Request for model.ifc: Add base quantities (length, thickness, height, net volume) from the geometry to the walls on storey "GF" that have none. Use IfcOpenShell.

First a look at what the model holds.

```python
import ifcopenshell
import ifcopenshell.util.element
import ifcopenshell.util.unit

model = ifcopenshell.open("model.ifc")
print(model.schema)
for unit_type in ("LENGTHUNIT", "AREAUNIT", "VOLUMEUNIT"):
    print(unit_type, ifcopenshell.util.unit.calculate_unit_scale(model, unit_type))
storey = next(s for s in model.by_type("IfcBuildingStorey") if s.Name == "GF")
walls = [e for e in ifcopenshell.util.element.get_decomposition(storey) if e.is_a("IfcWall")]
for e in sorted(walls, key=lambda e: e.id()):
    print(e.id(), e.is_a(), e.Name, list(ifcopenshell.util.element.get_psets(e, qtos_only=True)), sep=" | ")
```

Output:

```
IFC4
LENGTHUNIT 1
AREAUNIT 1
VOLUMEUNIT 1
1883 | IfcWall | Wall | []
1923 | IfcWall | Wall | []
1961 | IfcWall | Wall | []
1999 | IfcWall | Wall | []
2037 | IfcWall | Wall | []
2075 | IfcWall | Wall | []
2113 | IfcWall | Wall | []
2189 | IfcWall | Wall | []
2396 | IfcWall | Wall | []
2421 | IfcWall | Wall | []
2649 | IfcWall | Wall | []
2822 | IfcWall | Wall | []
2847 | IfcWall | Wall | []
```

```python
import ifcopenshell
import ifcopenshell.api.pset
import ifcopenshell.geom
import ifcopenshell.util.element
import ifcopenshell.util.shape
import ifcopenshell.util.unit

model = ifcopenshell.open("model.ifc")
unit_scale = ifcopenshell.util.unit.calculate_unit_scale(model)
volume_scale = ifcopenshell.util.unit.calculate_unit_scale(model, "VOLUMEUNIT")
settings = ifcopenshell.geom.settings()

storey = next(s for s in model.by_type("IfcBuildingStorey") if s.Name == "GF")
walls = [e for e in ifcopenshell.util.element.get_decomposition(storey) if e.is_a("IfcWall")]

for e in sorted(walls, key=lambda e: e.id()):
    if ifcopenshell.util.element.get_psets(e, qtos_only=True, should_inherit=False):
        continue
    # Geometry comes back in metres, in the element's own axes.
    shape = ifcopenshell.geom.create_shape(settings, e)
    values = {
        "Length": ifcopenshell.util.shape.get_x(shape.geometry) / unit_scale,
        "Width": ifcopenshell.util.shape.get_y(shape.geometry) / unit_scale,
        "Height": ifcopenshell.util.shape.get_z(shape.geometry) / unit_scale,
        "NetVolume": ifcopenshell.util.shape.get_volume(shape.geometry) / volume_scale,
    }
    qto = ifcopenshell.api.pset.add_qto(model, product=e, name="Qto_WallBaseQuantities")
    ifcopenshell.api.pset.edit_qto(model, qto=qto, properties=values)
    print(e.id(), {k: round(v, 3) for k, v in values.items()})

model.write("model-out.ifc")
```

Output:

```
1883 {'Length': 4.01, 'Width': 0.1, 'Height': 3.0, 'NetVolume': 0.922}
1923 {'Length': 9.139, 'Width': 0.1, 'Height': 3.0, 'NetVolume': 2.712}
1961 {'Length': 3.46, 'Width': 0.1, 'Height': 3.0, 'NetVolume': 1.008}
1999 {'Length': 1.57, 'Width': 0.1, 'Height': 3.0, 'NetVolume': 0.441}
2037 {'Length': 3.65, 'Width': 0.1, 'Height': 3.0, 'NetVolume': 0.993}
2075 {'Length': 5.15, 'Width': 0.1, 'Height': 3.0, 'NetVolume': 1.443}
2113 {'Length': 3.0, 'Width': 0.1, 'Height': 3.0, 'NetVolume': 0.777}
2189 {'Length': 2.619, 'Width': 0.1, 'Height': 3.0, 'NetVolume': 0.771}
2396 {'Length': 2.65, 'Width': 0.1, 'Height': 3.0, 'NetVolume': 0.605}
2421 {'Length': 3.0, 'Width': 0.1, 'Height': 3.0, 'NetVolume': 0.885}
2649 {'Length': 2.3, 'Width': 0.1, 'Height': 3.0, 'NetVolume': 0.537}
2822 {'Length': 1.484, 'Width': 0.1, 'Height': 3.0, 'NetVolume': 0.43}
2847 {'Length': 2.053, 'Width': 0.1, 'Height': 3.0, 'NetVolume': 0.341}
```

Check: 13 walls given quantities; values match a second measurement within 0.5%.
